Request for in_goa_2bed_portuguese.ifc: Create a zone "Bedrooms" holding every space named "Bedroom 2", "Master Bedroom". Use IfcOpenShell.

First a look at what the model holds.

```python
import ifcopenshell

model = ifcopenshell.open("in_goa_2bed_portuguese.ifc")
print(model.schema)
seen = {}
for space in model.by_type("IfcSpace"):
    seen[space.LongName] = seen.get(space.LongName, 0) + 1
for name, count in sorted(seen.items(), key=str):
    print(count, "x", name)
print("zones:", [z.Name for z in model.by_type("IfcZone")][:20])
```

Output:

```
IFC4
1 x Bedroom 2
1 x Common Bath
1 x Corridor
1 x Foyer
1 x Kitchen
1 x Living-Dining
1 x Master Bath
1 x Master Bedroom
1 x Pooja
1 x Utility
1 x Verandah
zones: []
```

```python
import ifcopenshell
import ifcopenshell.api.group
import ifcopenshell.api.root

model = ifcopenshell.open("in_goa_2bed_portuguese.ifc")

names = {"Bedroom 2", "Master Bedroom"}
spaces = [s for s in model.by_type("IfcSpace") if s.LongName in names]

zone = ifcopenshell.api.root.create_entity(model, ifc_class="IfcZone", name="Bedrooms")
ifcopenshell.api.group.assign_group(model, products=spaces, group=zone)
print(len(spaces), "spaces in", zone.Name)

model.write("in_goa_2bed_portuguese_rev.ifc")
```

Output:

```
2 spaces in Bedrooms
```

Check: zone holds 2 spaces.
